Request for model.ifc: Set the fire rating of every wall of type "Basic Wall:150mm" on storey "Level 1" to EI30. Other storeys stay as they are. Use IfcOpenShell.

First a look at what the model holds.

```python
import ifcopenshell
import ifcopenshell.util.element

model = ifcopenshell.open("model.ifc")
print(model.schema)
storey = next(s for s in model.by_type("IfcBuildingStorey") if s.Name == "Level 1")
walls = [e for e in ifcopenshell.util.element.get_decomposition(storey) if e.is_a("IfcWall")]
seen = {}
for e in walls:
    element_type = ifcopenshell.util.element.get_type(e)
    key = (element_type.Name if element_type != e and element_type else None, ifcopenshell.util.element.get_pset(e, "Pset_WallCommon", "FireRating"))
    seen[key] = seen.get(key, 0) + 1
for (name, value), count in sorted(seen.items(), key=str):
    print(count, "x", name, "|", value)
```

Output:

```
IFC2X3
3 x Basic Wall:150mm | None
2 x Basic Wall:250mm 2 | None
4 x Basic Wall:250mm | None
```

```python
import ifcopenshell
import ifcopenshell.api.pset
import ifcopenshell.util.element

model = ifcopenshell.open("model.ifc")

storey = next(s for s in model.by_type("IfcBuildingStorey") if s.Name == "Level 1")
walls = [e for e in ifcopenshell.util.element.get_decomposition(storey) if e.is_a("IfcWall")]

count = 0
for e in walls:
    element_type = ifcopenshell.util.element.get_type(e)
    if element_type in (None, e) or element_type.Name != "Basic Wall:150mm":
        continue
    # add_pset returns the element's existing set when there is one.
    pset = ifcopenshell.api.pset.add_pset(model, product=e, name="Pset_WallCommon")
    ifcopenshell.api.pset.edit_pset(model, pset=pset, properties={"FireRating": "EI30"})
    count += 1

print(count, "walls updated")

model.write("model_rev.ifc")
```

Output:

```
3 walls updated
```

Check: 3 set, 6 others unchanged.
